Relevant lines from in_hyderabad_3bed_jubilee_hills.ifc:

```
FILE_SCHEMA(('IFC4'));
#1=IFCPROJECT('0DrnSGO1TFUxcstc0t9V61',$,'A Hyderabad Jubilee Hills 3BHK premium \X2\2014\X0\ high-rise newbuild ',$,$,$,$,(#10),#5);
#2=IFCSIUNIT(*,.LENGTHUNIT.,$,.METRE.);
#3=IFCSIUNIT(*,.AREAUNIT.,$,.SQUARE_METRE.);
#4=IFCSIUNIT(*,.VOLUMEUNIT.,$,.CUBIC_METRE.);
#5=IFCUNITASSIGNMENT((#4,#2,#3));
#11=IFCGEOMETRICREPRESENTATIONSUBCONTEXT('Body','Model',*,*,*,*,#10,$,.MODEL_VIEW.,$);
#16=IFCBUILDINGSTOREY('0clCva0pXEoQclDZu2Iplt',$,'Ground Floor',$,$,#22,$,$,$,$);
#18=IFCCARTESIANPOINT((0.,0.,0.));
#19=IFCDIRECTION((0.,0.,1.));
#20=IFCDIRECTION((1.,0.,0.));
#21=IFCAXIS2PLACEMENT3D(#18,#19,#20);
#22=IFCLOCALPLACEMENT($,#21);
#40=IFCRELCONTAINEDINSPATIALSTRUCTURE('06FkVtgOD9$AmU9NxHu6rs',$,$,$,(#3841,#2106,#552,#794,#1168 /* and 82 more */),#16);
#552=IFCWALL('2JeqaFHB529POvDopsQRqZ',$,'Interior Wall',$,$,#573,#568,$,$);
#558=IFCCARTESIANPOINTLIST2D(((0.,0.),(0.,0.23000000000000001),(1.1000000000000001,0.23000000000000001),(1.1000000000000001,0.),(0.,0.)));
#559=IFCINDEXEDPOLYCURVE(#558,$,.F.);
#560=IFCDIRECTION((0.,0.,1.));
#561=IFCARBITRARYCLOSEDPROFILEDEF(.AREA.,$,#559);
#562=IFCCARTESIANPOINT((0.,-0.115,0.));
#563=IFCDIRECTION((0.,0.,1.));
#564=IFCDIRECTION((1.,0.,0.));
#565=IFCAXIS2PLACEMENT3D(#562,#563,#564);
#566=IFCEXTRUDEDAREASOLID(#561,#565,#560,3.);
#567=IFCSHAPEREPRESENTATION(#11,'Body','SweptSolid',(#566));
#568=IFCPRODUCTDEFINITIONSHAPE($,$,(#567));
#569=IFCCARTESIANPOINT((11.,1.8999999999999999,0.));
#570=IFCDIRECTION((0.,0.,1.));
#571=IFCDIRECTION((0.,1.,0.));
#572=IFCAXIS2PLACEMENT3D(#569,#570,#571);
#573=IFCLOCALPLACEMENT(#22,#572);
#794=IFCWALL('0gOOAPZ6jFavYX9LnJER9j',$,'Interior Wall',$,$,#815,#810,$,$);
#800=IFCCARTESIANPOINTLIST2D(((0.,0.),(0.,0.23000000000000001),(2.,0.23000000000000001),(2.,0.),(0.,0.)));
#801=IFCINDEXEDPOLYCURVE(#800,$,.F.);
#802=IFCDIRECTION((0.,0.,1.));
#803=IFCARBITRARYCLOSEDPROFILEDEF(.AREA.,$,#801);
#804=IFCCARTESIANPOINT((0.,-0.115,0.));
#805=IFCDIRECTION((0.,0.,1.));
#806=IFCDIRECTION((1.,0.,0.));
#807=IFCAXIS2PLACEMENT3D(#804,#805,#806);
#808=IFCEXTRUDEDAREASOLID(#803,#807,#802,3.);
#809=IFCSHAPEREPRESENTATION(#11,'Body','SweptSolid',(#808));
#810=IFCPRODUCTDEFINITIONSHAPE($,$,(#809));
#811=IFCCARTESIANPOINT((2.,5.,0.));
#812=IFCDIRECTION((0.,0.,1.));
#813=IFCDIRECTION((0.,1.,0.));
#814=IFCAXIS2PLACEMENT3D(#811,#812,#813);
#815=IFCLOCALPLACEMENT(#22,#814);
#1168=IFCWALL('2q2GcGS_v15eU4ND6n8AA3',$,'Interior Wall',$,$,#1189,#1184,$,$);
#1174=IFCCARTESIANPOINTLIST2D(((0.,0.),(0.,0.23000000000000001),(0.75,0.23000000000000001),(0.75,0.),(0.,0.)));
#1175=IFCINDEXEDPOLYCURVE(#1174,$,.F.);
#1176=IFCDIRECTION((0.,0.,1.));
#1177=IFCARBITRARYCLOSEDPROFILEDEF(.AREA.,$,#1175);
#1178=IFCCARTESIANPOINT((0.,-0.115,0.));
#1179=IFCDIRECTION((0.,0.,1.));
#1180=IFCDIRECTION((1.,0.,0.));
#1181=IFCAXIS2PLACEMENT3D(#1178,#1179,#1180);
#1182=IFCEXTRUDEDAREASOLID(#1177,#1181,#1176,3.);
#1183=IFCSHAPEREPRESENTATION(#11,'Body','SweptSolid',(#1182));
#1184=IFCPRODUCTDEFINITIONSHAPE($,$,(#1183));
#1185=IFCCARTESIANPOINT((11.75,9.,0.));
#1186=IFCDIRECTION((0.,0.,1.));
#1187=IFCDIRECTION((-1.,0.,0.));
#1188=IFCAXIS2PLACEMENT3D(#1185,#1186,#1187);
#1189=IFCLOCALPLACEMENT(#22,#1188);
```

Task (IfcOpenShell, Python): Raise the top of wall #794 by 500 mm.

```python
import ifcopenshell
import ifcopenshell.geom
import ifcopenshell.util.representation
import ifcopenshell.util.shape
import ifcopenshell.util.unit

model = ifcopenshell.open("in_hyderabad_3bed_jubilee_hills.ifc")
unit_scale = ifcopenshell.util.unit.calculate_unit_scale(model)
settings = ifcopenshell.geom.settings()


def volume(element):
    """Net volume in cubic metres, openings subtracted."""
    shape = ifcopenshell.geom.create_shape(settings, element)
    return ifcopenshell.util.shape.get_volume(shape.geometry)


wall = model.by_id(794)
before = volume(wall)

body = ifcopenshell.util.representation.get_representation(wall, "Model", "Body")
solid = body.Items[0]
old_height = solid.Depth
solid.Depth += 0.5 / unit_scale
after = volume(wall)

print(f"height {old_height:g} -> {solid.Depth:g}, volume {before:.3f} -> {after:.3f} m3")

model.write("in_hyderabad_3bed_jubilee_hills_rev.ifc")
```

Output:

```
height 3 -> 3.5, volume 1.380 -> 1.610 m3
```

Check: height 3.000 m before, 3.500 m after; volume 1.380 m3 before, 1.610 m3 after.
